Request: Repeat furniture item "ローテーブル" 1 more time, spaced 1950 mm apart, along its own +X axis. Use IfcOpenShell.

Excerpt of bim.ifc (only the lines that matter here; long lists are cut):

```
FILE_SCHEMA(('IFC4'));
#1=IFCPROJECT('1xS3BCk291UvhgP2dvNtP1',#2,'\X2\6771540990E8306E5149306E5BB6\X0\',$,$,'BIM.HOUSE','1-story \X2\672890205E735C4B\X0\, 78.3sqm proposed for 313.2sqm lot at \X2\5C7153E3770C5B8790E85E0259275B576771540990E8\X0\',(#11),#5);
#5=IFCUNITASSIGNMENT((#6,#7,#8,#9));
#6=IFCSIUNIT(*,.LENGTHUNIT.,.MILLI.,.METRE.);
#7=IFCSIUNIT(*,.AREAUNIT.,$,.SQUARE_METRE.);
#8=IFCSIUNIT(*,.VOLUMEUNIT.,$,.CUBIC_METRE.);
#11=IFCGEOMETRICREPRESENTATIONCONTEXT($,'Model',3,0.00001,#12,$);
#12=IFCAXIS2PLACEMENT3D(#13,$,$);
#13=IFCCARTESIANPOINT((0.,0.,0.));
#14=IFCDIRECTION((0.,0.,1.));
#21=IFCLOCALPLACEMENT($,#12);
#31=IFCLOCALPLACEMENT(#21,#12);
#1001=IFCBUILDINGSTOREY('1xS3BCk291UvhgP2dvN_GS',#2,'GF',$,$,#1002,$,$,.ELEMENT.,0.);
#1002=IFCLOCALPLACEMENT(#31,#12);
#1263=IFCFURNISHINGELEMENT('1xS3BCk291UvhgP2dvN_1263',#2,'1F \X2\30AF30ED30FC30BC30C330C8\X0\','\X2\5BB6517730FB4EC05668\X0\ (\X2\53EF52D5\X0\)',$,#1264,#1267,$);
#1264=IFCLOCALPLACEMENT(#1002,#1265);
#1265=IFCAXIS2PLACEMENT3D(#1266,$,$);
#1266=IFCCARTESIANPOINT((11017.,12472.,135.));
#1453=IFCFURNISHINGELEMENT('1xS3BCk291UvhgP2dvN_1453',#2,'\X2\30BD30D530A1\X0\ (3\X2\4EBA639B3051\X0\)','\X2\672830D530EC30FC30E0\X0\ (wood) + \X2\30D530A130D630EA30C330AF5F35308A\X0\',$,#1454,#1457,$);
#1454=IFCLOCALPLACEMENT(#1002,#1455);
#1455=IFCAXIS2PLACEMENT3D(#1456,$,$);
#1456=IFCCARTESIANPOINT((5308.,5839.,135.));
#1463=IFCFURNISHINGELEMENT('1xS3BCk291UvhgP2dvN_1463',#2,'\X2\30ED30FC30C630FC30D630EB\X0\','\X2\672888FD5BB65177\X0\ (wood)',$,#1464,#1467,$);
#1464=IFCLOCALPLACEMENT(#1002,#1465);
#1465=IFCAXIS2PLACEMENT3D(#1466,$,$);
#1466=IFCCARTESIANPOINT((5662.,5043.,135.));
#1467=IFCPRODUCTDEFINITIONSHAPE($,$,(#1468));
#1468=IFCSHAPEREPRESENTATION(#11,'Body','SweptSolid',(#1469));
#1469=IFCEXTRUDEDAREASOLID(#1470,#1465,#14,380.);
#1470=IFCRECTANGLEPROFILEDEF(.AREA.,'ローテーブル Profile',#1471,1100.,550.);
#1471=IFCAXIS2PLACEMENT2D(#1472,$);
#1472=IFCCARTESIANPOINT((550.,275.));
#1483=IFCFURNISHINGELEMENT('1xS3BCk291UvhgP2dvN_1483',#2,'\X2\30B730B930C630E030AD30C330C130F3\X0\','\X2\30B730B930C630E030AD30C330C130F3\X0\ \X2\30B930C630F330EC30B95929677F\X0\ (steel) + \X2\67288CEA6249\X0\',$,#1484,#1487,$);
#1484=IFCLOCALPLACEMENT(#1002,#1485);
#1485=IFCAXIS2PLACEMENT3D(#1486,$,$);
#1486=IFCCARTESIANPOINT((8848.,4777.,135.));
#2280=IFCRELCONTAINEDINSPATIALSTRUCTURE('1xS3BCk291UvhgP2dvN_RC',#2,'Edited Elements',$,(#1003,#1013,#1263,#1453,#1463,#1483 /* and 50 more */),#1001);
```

```python
import ifcopenshell
import ifcopenshell.api.geometry
import ifcopenshell.api.root
import ifcopenshell.util.element
import ifcopenshell.util.placement
import ifcopenshell.util.unit

model = ifcopenshell.open("bim.ifc")
unit_scale = ifcopenshell.util.unit.calculate_unit_scale(model)


def reuse_history(source, copy):
    """copy_class also copies each property set's owner history, people and application; keep the originals."""
    for rel in copy.IsDefinedBy:
        if rel.is_a("IfcRelDefinesByProperties") and (history := rel.RelatingPropertyDefinition.OwnerHistory):
            rel.RelatingPropertyDefinition.OwnerHistory = source.OwnerHistory
            ifcopenshell.util.element.remove_deep2(model, history)


source = model.by_guid("1xS3BCk291UvhgP2dvN_1463")
base = ifcopenshell.util.placement.get_local_placement(source.ObjectPlacement)
step = base[:3, 0] * 1.95 / unit_scale

for i in range(1, 2):
    copy = ifcopenshell.api.root.copy_class(model, product=source)
    copy.Representation = ifcopenshell.util.element.copy_deep(
        model, source.Representation, exclude=["IfcGeometricRepresentationContext", "IfcRepresentationMap"]
    )
    reuse_history(source, copy)
    matrix = base.copy()
    matrix[:3, 3] += i * step
    print("added at", matrix[:3, 3].round(3) + 0.0)
    ifcopenshell.api.geometry.edit_object_placement(model, product=copy, matrix=matrix, is_si=False)

model.write("bim-out.ifc")
```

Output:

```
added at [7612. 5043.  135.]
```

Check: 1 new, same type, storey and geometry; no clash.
